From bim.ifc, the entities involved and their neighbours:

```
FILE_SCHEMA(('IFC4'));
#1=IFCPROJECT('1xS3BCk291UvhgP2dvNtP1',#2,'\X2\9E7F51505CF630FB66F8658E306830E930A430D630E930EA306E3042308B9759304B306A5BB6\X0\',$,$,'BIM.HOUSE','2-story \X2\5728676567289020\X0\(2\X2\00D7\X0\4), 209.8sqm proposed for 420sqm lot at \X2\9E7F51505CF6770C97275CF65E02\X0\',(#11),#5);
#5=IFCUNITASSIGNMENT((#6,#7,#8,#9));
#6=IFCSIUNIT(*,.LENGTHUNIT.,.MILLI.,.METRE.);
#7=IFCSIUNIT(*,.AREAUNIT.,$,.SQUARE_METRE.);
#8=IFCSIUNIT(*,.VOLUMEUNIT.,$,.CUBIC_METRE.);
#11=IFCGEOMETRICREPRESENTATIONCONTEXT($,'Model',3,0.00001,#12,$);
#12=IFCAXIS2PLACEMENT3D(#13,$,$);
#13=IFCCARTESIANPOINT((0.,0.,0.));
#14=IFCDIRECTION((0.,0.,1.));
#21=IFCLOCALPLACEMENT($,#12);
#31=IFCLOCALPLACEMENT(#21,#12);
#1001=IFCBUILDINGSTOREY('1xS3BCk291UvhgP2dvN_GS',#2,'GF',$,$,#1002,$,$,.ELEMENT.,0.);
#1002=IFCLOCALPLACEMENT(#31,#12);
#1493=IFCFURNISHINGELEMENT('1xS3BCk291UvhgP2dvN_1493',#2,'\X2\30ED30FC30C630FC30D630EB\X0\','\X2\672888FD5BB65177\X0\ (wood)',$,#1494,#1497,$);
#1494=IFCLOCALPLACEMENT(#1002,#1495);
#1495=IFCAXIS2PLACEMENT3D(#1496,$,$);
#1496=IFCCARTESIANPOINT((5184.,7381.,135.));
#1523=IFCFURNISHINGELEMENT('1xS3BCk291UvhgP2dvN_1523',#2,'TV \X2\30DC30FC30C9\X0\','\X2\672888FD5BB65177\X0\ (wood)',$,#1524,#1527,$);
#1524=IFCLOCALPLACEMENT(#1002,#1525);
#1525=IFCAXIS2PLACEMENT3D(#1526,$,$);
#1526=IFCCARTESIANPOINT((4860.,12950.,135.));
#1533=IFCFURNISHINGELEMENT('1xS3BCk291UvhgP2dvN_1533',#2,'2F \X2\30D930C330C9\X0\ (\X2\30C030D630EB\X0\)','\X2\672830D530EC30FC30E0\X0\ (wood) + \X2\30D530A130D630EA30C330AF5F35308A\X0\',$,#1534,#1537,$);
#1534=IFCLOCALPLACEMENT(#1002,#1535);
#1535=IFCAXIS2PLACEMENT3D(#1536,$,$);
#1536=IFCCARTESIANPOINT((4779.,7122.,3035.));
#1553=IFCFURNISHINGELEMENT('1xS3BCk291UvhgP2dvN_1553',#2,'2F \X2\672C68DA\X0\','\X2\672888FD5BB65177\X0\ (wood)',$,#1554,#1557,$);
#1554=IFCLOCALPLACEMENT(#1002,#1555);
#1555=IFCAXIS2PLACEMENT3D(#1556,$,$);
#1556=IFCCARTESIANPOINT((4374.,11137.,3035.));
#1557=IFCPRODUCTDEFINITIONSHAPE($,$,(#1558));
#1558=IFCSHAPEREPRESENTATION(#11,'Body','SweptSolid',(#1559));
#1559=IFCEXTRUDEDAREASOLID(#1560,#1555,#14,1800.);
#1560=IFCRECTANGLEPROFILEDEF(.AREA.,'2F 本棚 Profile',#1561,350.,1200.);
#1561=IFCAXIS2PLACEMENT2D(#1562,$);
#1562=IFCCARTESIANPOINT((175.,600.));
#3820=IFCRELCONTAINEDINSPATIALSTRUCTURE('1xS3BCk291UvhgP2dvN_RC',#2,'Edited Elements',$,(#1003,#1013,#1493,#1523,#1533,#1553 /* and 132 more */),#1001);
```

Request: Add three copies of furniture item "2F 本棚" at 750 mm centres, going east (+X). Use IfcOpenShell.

```python
import numpy as np
import ifcopenshell
import ifcopenshell.api.geometry
import ifcopenshell.api.root
import ifcopenshell.util.element
import ifcopenshell.util.placement

model = ifcopenshell.open("bim.ifc")


def reuse_history(source, copy):
    """copy_class also copies each property set's owner history, people and application; keep the originals."""
    for rel in copy.IsDefinedBy:
        if rel.is_a("IfcRelDefinesByProperties") and (history := rel.RelatingPropertyDefinition.OwnerHistory):
            rel.RelatingPropertyDefinition.OwnerHistory = source.OwnerHistory
            ifcopenshell.util.element.remove_deep2(model, history)


source = model.by_guid("1xS3BCk291UvhgP2dvN_1553")
base = ifcopenshell.util.placement.get_local_placement(source.ObjectPlacement)
step = np.array([1.0, 0.0, 0.0]) * 750.0

for i in range(1, 4):
    copy = ifcopenshell.api.root.copy_class(model, product=source)
    copy.Representation = ifcopenshell.util.element.copy_deep(
        model, source.Representation, exclude=["IfcGeometricRepresentationContext", "IfcRepresentationMap"]
    )
    reuse_history(source, copy)
    matrix = base.copy()
    matrix[:3, 3] += i * step
    print("added at", matrix[:3, 3].round(3) + 0.0)
    ifcopenshell.api.geometry.edit_object_placement(model, product=copy, matrix=matrix, is_si=False)

model.write("bim_edited.ifc")
```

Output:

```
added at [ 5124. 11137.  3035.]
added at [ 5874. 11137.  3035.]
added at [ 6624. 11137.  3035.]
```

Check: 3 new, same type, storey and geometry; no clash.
